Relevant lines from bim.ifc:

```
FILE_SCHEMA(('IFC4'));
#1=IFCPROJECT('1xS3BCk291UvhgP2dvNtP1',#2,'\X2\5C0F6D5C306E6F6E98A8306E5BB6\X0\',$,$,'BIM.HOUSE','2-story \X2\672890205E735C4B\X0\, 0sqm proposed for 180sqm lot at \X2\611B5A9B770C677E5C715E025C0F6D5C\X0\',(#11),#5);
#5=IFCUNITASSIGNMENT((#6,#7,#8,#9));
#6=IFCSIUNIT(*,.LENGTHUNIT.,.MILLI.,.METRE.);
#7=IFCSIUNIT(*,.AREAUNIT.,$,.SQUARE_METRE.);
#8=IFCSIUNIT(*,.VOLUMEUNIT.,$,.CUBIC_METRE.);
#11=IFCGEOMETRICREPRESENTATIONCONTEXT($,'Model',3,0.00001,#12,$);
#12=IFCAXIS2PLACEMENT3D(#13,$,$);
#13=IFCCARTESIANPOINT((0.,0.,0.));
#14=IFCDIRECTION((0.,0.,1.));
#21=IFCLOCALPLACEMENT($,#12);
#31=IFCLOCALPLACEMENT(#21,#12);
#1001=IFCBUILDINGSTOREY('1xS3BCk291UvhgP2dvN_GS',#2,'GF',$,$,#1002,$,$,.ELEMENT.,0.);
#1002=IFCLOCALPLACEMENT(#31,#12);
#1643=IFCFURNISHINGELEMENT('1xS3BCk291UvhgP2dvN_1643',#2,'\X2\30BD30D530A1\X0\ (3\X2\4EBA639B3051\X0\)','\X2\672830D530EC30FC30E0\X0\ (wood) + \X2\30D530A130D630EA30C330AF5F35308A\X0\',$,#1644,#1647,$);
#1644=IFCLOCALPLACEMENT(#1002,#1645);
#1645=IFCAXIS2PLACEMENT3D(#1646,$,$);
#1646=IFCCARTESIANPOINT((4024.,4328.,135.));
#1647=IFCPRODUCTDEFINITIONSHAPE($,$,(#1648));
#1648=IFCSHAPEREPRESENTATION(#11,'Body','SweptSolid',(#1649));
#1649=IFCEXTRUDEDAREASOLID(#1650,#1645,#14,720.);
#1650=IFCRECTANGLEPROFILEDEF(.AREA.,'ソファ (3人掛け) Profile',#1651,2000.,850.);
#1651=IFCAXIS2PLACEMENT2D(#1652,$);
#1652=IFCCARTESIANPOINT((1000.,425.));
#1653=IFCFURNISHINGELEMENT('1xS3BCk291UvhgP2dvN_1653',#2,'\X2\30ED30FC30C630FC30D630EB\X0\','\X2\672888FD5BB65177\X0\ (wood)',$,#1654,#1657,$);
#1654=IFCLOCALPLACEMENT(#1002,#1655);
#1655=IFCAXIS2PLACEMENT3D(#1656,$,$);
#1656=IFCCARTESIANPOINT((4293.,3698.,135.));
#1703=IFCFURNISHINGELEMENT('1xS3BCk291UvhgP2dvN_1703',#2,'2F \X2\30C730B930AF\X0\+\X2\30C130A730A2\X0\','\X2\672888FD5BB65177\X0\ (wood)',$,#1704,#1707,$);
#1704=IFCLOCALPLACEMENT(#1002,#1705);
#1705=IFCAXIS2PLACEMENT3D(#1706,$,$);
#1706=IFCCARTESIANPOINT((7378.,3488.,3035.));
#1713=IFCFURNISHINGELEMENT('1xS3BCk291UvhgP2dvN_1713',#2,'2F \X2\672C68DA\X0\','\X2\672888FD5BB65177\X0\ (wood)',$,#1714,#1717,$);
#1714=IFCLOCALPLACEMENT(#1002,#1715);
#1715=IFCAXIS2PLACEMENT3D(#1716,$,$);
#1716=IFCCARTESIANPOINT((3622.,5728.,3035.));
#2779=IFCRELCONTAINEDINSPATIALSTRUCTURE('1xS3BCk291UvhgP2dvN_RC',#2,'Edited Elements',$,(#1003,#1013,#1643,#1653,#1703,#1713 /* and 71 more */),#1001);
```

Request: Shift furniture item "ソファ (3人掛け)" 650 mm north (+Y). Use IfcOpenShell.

```python
import ifcopenshell
import ifcopenshell.api.geometry
import ifcopenshell.util.placement
import ifcopenshell.util.unit

model = ifcopenshell.open("bim.ifc")
unit_scale = ifcopenshell.util.unit.calculate_unit_scale(model)

item = model.by_id(1643)
matrix = ifcopenshell.util.placement.get_local_placement(item.ObjectPlacement)
matrix[1, 3] += 0.65 / unit_scale
ifcopenshell.api.geometry.edit_object_placement(model, product=item, matrix=matrix, is_si=False)

print(ifcopenshell.util.placement.get_local_placement(item.ObjectPlacement).round(3) + 0.0)

model.write("bim_updated.ifc")
```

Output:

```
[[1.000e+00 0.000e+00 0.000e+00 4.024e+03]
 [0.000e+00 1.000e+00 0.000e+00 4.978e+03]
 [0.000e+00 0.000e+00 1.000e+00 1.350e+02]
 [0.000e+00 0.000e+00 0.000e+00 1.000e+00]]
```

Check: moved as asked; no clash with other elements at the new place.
